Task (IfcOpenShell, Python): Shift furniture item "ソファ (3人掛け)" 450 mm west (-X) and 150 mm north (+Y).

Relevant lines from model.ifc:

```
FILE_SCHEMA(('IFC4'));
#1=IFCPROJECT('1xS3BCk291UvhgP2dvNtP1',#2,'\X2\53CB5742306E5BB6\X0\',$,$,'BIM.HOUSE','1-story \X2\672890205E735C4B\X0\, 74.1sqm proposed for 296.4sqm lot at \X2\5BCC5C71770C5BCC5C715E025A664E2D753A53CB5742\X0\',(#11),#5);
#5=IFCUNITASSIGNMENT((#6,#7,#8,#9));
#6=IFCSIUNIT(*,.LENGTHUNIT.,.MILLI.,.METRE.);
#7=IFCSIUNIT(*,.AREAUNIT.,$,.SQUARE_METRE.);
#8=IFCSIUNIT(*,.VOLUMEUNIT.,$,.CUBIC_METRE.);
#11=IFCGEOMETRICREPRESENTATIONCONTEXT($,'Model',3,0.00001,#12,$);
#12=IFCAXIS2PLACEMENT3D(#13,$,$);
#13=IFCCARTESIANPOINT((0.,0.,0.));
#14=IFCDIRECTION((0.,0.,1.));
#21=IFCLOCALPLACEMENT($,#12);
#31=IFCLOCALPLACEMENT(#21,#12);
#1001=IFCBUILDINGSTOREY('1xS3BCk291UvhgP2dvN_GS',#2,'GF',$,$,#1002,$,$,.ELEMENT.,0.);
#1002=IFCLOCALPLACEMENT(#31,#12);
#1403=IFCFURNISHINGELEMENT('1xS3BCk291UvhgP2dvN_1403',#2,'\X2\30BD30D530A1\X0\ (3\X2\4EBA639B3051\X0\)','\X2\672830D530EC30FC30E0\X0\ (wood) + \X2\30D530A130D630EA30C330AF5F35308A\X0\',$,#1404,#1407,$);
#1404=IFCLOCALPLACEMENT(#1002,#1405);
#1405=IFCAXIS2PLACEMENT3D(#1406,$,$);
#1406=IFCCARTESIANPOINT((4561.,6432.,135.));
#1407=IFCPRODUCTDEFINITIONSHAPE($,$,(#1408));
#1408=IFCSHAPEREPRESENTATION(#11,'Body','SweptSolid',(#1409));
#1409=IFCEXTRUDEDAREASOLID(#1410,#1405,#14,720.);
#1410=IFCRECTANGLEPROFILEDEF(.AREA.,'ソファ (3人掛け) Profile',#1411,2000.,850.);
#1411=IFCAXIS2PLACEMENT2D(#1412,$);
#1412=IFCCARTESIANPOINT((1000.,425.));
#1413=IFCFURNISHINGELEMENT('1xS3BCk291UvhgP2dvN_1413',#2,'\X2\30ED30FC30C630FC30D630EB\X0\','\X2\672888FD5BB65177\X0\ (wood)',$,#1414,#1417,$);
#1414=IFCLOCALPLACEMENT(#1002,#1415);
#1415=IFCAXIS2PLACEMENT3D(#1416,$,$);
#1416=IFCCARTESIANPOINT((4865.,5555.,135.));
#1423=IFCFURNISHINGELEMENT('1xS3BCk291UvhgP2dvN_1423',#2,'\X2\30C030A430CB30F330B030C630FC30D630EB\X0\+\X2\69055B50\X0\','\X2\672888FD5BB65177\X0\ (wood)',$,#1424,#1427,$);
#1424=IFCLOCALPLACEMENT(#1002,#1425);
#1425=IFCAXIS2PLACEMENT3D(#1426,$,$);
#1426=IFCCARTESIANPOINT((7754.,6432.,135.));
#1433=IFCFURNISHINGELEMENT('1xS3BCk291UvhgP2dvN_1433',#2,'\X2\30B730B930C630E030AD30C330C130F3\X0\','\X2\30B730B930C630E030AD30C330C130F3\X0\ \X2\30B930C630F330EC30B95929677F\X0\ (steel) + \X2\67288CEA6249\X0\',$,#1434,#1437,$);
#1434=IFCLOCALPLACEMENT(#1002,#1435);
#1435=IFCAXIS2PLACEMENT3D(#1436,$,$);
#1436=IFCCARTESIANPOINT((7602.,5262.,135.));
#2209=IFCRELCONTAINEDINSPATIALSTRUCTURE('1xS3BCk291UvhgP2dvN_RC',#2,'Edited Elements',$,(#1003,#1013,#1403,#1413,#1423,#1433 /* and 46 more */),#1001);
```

```python
import ifcopenshell
import ifcopenshell.api.geometry
import ifcopenshell.util.placement
import ifcopenshell.util.unit

model = ifcopenshell.open("model.ifc")
unit_scale = ifcopenshell.util.unit.calculate_unit_scale(model)

item = model.by_id(1403)
matrix = ifcopenshell.util.placement.get_local_placement(item.ObjectPlacement)
matrix[0, 3] -= 0.45 / unit_scale
matrix[1, 3] += 0.15 / unit_scale
ifcopenshell.api.geometry.edit_object_placement(model, product=item, matrix=matrix, is_si=False)

print(ifcopenshell.util.placement.get_local_placement(item.ObjectPlacement).round(3) + 0.0)

model.write("model_updated.ifc")
```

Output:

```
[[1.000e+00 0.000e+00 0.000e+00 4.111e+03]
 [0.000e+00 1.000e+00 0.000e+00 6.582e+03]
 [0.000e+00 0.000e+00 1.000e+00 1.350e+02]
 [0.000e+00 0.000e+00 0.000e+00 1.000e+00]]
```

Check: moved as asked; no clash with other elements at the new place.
